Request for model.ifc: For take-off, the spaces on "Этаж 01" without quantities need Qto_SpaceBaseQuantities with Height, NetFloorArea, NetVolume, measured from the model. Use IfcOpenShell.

First a look at what the model holds.

```python
import ifcopenshell
import ifcopenshell.util.element
import ifcopenshell.util.unit

model = ifcopenshell.open("model.ifc")
print(model.schema)
for unit_type in ("LENGTHUNIT", "AREAUNIT", "VOLUMEUNIT"):
    print(unit_type, ifcopenshell.util.unit.calculate_unit_scale(model, unit_type))
storey = next(s for s in model.by_type("IfcBuildingStorey") if s.Name == "Этаж 01")
spaces = [e for e in ifcopenshell.util.element.get_decomposition(storey) if e.is_a("IfcSpace")]
for e in sorted(spaces, key=lambda e: e.id()):
    print(e.id(), e.is_a(), e.Name, list(ifcopenshell.util.element.get_psets(e, qtos_only=True)), sep=" | ")
```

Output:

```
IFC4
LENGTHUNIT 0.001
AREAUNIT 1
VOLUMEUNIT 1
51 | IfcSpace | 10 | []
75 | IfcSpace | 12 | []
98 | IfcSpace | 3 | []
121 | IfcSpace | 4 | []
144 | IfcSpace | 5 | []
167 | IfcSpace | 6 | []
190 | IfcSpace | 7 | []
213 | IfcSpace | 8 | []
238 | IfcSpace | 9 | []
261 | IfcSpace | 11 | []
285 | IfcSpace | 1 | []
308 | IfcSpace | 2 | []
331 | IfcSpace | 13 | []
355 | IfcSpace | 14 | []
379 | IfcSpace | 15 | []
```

```python
import ifcopenshell
import ifcopenshell.api.pset
import ifcopenshell.geom
import ifcopenshell.util.element
import ifcopenshell.util.shape
import ifcopenshell.util.unit

model = ifcopenshell.open("model.ifc")
unit_scale = ifcopenshell.util.unit.calculate_unit_scale(model)
area_scale = ifcopenshell.util.unit.calculate_unit_scale(model, "AREAUNIT")
volume_scale = ifcopenshell.util.unit.calculate_unit_scale(model, "VOLUMEUNIT")
settings = ifcopenshell.geom.settings()

storey = next(s for s in model.by_type("IfcBuildingStorey") if s.Name == "Этаж 01")
spaces = [e for e in ifcopenshell.util.element.get_decomposition(storey) if e.is_a("IfcSpace")]

for e in sorted(spaces, key=lambda e: e.id()):
    if ifcopenshell.util.element.get_psets(e, qtos_only=True, should_inherit=False):
        continue
    # Geometry comes back in metres, in the element's own axes.
    shape = ifcopenshell.geom.create_shape(settings, e)
    values = {
        "Height": ifcopenshell.util.shape.get_z(shape.geometry) / unit_scale,
        "NetFloorArea": ifcopenshell.util.shape.get_footprint_area(shape.geometry) / area_scale,
        "NetVolume": ifcopenshell.util.shape.get_volume(shape.geometry) / volume_scale,
    }
    qto = ifcopenshell.api.pset.add_qto(model, product=e, name="Qto_SpaceBaseQuantities")
    ifcopenshell.api.pset.edit_qto(model, qto=qto, properties=values)
    print(e.id(), {k: round(v, 3) for k, v in values.items()})

model.write("model_edited.ifc")
```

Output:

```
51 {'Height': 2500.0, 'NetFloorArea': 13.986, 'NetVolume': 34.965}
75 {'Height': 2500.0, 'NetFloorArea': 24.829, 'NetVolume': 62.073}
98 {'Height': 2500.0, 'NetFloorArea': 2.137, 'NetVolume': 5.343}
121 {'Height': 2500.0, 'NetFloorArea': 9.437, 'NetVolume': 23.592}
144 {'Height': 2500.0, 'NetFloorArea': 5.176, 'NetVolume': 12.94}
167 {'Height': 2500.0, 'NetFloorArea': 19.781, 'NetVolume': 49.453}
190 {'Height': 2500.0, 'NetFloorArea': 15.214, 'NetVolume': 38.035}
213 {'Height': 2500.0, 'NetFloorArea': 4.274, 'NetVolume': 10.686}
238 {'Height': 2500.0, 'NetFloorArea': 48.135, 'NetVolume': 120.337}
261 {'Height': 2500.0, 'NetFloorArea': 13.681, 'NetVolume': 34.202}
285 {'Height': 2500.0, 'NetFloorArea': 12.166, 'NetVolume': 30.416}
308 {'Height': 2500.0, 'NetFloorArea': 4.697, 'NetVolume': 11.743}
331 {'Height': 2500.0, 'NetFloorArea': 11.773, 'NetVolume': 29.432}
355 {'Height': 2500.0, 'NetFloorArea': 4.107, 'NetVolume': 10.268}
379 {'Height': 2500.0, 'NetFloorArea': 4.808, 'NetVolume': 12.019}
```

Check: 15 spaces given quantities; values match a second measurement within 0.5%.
